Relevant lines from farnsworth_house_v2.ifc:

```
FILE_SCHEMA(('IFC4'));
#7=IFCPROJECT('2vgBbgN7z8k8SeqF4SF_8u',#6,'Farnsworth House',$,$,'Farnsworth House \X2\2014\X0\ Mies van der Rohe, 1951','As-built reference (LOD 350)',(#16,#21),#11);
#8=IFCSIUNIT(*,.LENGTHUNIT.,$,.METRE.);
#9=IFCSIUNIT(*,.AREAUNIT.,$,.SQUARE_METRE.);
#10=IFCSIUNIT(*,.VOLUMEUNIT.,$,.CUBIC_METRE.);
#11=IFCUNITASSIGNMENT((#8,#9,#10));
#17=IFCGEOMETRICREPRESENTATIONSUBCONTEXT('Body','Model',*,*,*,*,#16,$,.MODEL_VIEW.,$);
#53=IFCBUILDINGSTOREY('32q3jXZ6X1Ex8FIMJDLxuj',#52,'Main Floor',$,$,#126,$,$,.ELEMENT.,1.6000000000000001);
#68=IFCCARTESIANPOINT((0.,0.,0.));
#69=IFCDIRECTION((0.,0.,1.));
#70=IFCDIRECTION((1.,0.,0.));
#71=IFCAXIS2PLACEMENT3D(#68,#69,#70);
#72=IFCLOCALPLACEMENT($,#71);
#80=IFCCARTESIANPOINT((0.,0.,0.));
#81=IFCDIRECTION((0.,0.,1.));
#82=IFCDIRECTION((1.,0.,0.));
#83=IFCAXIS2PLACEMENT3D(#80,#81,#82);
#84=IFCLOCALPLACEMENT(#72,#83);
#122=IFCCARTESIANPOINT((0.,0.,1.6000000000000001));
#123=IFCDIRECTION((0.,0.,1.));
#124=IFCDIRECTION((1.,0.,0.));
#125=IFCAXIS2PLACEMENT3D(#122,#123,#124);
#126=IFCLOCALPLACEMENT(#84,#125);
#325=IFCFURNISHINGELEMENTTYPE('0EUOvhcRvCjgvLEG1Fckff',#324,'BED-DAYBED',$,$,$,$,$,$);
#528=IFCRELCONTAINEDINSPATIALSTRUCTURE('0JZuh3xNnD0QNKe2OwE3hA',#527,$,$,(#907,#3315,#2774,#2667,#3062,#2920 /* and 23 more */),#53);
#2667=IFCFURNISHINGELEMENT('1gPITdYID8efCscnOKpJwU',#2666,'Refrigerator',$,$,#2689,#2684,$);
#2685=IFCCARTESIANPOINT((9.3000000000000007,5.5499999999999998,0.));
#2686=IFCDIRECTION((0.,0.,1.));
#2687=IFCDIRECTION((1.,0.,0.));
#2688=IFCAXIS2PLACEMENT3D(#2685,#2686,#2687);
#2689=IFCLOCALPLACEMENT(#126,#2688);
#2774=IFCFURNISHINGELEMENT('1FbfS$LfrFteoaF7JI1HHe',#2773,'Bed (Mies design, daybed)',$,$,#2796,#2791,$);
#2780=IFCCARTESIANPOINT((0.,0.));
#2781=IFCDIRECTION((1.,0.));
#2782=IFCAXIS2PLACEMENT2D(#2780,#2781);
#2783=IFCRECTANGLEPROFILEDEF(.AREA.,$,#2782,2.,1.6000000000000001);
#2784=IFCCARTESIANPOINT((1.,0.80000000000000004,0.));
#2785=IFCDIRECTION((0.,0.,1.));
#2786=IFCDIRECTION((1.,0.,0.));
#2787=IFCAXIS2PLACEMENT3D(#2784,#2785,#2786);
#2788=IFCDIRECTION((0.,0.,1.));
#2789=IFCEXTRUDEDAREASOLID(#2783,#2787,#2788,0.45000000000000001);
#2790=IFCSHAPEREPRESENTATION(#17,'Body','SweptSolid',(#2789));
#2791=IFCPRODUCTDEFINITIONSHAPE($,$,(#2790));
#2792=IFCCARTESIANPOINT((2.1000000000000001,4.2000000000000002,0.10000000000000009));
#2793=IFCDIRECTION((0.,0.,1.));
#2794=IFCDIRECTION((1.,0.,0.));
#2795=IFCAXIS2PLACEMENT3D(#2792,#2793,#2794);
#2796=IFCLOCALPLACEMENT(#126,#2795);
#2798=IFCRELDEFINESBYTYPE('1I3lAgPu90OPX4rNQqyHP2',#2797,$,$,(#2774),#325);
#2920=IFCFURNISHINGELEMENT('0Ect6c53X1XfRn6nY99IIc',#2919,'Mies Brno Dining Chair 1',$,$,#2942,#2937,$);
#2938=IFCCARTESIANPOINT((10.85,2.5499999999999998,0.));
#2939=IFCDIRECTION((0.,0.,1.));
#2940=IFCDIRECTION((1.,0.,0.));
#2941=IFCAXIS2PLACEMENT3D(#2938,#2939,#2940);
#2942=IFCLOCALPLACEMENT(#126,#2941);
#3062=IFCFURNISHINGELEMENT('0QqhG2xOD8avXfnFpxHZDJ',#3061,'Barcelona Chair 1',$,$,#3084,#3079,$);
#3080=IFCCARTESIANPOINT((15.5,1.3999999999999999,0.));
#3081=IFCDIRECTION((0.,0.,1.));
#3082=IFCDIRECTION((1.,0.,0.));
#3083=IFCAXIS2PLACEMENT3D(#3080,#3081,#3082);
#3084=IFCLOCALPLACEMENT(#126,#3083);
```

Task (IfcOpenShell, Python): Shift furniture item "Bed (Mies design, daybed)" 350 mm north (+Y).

```python
import ifcopenshell
import ifcopenshell.api.geometry
import ifcopenshell.util.placement
import ifcopenshell.util.unit

model = ifcopenshell.open("farnsworth_house_v2.ifc")
unit_scale = ifcopenshell.util.unit.calculate_unit_scale(model)

item = model.by_guid("1FbfS$LfrFteoaF7JI1HHe")
matrix = ifcopenshell.util.placement.get_local_placement(item.ObjectPlacement)
matrix[1, 3] += 0.35 / unit_scale
ifcopenshell.api.geometry.edit_object_placement(model, product=item, matrix=matrix, is_si=False)

print(ifcopenshell.util.placement.get_local_placement(item.ObjectPlacement).round(3) + 0.0)

model.write("farnsworth_house_v2_edited.ifc")
```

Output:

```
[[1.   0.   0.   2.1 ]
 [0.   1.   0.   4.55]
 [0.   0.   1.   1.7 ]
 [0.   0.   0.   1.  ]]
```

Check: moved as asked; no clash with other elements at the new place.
